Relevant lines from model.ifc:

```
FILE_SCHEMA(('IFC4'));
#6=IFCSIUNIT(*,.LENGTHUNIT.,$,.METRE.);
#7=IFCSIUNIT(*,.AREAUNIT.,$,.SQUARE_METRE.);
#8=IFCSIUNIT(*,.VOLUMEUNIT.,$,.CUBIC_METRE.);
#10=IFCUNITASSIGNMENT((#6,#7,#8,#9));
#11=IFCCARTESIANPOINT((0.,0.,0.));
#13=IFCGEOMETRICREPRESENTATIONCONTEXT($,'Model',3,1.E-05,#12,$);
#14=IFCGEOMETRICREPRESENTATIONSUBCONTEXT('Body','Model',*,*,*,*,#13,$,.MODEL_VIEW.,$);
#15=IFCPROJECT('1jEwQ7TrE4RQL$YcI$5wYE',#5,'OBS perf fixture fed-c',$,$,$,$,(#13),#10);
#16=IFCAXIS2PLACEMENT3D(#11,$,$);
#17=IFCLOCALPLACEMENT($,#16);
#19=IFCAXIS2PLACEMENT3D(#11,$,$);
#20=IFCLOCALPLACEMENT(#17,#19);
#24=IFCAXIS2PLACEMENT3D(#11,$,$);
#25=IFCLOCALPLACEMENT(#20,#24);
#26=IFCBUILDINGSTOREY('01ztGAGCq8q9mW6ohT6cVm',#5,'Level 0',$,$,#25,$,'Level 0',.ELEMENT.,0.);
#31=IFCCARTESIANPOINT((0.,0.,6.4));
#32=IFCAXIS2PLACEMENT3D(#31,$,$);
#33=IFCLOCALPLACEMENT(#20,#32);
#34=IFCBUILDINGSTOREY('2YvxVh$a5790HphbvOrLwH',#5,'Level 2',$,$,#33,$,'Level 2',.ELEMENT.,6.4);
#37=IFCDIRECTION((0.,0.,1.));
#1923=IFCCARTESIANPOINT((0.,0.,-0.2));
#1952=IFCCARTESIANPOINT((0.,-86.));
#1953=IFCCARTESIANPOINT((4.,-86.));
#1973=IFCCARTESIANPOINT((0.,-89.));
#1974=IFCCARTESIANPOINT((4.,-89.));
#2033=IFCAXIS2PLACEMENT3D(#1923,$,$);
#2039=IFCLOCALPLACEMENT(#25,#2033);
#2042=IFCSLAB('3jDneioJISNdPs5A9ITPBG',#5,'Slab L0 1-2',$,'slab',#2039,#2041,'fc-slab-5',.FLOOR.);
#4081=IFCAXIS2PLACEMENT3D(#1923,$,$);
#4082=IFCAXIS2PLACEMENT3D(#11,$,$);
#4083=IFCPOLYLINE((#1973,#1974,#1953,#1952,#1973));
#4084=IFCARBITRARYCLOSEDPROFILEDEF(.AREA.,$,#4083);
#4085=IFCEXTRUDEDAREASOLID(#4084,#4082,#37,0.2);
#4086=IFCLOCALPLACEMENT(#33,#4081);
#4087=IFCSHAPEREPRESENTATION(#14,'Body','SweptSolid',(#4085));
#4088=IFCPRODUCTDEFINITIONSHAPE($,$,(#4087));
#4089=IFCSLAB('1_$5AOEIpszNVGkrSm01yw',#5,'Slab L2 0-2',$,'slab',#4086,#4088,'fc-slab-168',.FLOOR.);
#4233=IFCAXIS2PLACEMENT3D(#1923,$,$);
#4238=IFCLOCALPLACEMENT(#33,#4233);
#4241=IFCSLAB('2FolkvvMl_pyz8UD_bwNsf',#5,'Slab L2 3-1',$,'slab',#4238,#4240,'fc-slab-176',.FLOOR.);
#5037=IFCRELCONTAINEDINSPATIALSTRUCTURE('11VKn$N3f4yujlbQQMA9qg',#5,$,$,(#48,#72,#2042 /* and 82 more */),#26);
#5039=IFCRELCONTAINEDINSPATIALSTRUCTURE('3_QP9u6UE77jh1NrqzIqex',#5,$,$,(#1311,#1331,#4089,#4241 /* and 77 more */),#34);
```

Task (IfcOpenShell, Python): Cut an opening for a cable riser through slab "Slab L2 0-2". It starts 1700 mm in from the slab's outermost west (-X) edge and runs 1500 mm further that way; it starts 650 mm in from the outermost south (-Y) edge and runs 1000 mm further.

```python
import numpy as np
import ifcopenshell
import ifcopenshell.api.feature
import ifcopenshell.api.geometry
import ifcopenshell.api.root
import ifcopenshell.geom
import ifcopenshell.util.placement
import ifcopenshell.util.representation
import ifcopenshell.util.shape
import ifcopenshell.util.unit

model = ifcopenshell.open("model.ifc")
unit_scale = ifcopenshell.util.unit.calculate_unit_scale(model)
settings = ifcopenshell.geom.settings()


def volume(element):
    """Net volume in cubic metres, openings subtracted."""
    shape = ifcopenshell.geom.create_shape(settings, element)
    return ifcopenshell.util.shape.get_volume(shape.geometry)


slab = model.by_guid("1_$5AOEIpszNVGkrSm01yw")
before = volume(slab)

# Extent in the slab's own axes, in metres. The edges named are its -X and -Y sides.
slab_shape = ifcopenshell.geom.create_shape(settings, slab)
vertices = ifcopenshell.util.shape.get_vertices(slab_shape.geometry)
x_min, y_min, bottom = vertices.min(axis=0)
top = vertices[:, 2].max()

opening = ifcopenshell.api.root.create_entity(model, ifc_class="IfcOpeningElement", name="Cable riser opening", predefined_type="OPENING")
context = ifcopenshell.util.representation.get_context(model, "Model", "Body", "MODEL_VIEW")
width, depth = 1.5, 1
outline = [(0.0, 0.0), (width, 0.0), (width, depth), (0.0, depth), (0.0, 0.0)]
# Overshoot both faces by 50 mm so the cut is clean.
shape = ifcopenshell.api.geometry.add_slab_representation(
    model, context=context, depth=top - bottom + 0.1, polyline=outline
)
ifcopenshell.api.geometry.assign_representation(model, product=opening, representation=shape)

matrix = ifcopenshell.util.placement.get_local_placement(slab.ObjectPlacement)
matrix[:, 3] = matrix @ np.append(np.array([x_min + 1.7, y_min + 0.65, bottom - 0.05]) / unit_scale, 1.0)
ifcopenshell.api.geometry.edit_object_placement(model, product=opening, matrix=matrix, is_si=False)
ifcopenshell.api.feature.add_feature(model, feature=opening, element=slab)

after = volume(slab)

print(f"slab volume {before:.3f} -> {after:.3f} m3")

model.write("model_v2.ifc")
```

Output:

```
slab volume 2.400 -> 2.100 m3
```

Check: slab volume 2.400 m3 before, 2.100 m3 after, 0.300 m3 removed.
